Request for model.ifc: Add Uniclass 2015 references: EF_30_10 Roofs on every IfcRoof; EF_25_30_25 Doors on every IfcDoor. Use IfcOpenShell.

First a look at what the model holds.

```python
import ifcopenshell

model = ifcopenshell.open("model.ifc")
print(model.schema)
print("classifications:", [c.Name for c in model.by_type("IfcClassification")])
for ifc_class in ("IfcDoor", "IfcRoof", "IfcStair", "IfcWall", "IfcWindow"):
    print(ifc_class, len(model.by_type(ifc_class)))
```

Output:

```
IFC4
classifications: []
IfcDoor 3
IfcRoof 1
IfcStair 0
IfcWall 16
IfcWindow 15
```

```python
import ifcopenshell
import ifcopenshell.api.classification

model = ifcopenshell.open("model.ifc")

system = ifcopenshell.api.classification.add_classification(model, classification="Uniclass 2015")

codes = {
    "IfcRoof": ("EF_30_10", "Roofs"),
    "IfcDoor": ("EF_25_30_25", "Doors"),
}
for ifc_class, (code, name) in codes.items():
    products = model.by_type(ifc_class)
    ifcopenshell.api.classification.add_reference(
        model, products=products, classification=system, identification=code, name=name
    )
    print(code, len(products))

model.write("model_rev.ifc")
```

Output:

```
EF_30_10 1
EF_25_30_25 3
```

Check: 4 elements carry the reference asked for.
